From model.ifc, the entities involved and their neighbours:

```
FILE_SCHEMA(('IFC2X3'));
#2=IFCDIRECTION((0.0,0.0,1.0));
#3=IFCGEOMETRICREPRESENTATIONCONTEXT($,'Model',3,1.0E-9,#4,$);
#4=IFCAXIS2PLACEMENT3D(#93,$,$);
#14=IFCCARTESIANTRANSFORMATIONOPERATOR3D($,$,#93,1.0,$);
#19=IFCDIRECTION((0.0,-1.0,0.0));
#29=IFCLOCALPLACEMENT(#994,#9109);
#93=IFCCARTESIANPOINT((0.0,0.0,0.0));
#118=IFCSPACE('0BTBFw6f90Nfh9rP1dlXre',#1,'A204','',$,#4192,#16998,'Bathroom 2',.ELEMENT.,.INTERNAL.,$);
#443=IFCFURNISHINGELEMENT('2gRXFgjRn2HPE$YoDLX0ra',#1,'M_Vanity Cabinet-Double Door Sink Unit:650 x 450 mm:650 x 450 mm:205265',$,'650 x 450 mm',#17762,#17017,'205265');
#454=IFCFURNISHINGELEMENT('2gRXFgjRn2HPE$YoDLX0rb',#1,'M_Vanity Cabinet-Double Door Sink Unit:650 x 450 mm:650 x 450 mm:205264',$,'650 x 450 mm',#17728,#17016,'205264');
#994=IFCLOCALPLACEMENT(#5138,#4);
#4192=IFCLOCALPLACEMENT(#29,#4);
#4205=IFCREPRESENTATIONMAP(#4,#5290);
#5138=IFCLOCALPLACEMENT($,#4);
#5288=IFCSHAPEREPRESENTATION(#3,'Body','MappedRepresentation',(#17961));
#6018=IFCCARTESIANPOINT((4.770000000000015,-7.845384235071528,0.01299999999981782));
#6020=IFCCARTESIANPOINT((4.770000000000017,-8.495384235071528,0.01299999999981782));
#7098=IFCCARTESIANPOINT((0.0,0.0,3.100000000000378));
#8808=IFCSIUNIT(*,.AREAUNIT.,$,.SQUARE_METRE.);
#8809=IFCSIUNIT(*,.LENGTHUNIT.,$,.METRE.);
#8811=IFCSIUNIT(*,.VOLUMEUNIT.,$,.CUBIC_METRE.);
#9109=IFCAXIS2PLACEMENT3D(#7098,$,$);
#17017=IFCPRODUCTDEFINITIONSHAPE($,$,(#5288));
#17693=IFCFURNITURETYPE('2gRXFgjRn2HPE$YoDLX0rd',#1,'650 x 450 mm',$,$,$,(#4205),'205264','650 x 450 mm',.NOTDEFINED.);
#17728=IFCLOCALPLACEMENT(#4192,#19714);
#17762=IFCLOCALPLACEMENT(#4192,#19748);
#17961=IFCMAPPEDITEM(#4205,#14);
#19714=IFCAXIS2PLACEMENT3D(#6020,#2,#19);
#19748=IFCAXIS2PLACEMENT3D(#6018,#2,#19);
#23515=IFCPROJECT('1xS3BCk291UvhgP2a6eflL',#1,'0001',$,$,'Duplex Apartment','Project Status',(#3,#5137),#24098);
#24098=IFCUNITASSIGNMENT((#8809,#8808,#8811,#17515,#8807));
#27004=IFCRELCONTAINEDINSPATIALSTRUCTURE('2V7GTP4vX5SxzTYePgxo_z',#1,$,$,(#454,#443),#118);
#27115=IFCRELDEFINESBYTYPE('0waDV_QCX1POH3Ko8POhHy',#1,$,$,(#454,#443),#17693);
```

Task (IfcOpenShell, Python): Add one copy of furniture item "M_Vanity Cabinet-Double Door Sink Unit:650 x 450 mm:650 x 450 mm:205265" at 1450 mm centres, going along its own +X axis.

```python
import ifcopenshell
import ifcopenshell.api.geometry
import ifcopenshell.api.root
import ifcopenshell.util.element
import ifcopenshell.util.placement

model = ifcopenshell.open("model.ifc")


def reuse_history(source, copy):
    """copy_class also copies each property set's owner history, people and application; keep the originals."""
    for rel in copy.IsDefinedBy:
        if rel.is_a("IfcRelDefinesByProperties") and (history := rel.RelatingPropertyDefinition.OwnerHistory):
            rel.RelatingPropertyDefinition.OwnerHistory = source.OwnerHistory
            ifcopenshell.util.element.remove_deep2(model, history)


source = model.by_guid("2gRXFgjRn2HPE$YoDLX0ra")
base = ifcopenshell.util.placement.get_local_placement(source.ObjectPlacement)
step = base[:3, 0] * 1.45

for i in range(1, 2):
    copy = ifcopenshell.api.root.copy_class(model, product=source)
    copy.Representation = ifcopenshell.util.element.copy_deep(
        model, source.Representation, exclude=["IfcGeometricRepresentationContext", "IfcRepresentationMap"]
    )
    copy.Name = "M_Vanity Cabinet-Double Door Sink Unit:650 x 450 mm:650 x 450 mm"
    copy.Tag = None
    reuse_history(source, copy)
    matrix = base.copy()
    matrix[:3, 3] += i * step
    print("added at", matrix[:3, 3].round(3) + 0.0)
    ifcopenshell.api.geometry.edit_object_placement(model, product=copy, matrix=matrix, is_si=False)

model.write("model-out.ifc")
```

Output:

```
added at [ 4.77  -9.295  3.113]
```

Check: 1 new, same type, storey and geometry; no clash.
